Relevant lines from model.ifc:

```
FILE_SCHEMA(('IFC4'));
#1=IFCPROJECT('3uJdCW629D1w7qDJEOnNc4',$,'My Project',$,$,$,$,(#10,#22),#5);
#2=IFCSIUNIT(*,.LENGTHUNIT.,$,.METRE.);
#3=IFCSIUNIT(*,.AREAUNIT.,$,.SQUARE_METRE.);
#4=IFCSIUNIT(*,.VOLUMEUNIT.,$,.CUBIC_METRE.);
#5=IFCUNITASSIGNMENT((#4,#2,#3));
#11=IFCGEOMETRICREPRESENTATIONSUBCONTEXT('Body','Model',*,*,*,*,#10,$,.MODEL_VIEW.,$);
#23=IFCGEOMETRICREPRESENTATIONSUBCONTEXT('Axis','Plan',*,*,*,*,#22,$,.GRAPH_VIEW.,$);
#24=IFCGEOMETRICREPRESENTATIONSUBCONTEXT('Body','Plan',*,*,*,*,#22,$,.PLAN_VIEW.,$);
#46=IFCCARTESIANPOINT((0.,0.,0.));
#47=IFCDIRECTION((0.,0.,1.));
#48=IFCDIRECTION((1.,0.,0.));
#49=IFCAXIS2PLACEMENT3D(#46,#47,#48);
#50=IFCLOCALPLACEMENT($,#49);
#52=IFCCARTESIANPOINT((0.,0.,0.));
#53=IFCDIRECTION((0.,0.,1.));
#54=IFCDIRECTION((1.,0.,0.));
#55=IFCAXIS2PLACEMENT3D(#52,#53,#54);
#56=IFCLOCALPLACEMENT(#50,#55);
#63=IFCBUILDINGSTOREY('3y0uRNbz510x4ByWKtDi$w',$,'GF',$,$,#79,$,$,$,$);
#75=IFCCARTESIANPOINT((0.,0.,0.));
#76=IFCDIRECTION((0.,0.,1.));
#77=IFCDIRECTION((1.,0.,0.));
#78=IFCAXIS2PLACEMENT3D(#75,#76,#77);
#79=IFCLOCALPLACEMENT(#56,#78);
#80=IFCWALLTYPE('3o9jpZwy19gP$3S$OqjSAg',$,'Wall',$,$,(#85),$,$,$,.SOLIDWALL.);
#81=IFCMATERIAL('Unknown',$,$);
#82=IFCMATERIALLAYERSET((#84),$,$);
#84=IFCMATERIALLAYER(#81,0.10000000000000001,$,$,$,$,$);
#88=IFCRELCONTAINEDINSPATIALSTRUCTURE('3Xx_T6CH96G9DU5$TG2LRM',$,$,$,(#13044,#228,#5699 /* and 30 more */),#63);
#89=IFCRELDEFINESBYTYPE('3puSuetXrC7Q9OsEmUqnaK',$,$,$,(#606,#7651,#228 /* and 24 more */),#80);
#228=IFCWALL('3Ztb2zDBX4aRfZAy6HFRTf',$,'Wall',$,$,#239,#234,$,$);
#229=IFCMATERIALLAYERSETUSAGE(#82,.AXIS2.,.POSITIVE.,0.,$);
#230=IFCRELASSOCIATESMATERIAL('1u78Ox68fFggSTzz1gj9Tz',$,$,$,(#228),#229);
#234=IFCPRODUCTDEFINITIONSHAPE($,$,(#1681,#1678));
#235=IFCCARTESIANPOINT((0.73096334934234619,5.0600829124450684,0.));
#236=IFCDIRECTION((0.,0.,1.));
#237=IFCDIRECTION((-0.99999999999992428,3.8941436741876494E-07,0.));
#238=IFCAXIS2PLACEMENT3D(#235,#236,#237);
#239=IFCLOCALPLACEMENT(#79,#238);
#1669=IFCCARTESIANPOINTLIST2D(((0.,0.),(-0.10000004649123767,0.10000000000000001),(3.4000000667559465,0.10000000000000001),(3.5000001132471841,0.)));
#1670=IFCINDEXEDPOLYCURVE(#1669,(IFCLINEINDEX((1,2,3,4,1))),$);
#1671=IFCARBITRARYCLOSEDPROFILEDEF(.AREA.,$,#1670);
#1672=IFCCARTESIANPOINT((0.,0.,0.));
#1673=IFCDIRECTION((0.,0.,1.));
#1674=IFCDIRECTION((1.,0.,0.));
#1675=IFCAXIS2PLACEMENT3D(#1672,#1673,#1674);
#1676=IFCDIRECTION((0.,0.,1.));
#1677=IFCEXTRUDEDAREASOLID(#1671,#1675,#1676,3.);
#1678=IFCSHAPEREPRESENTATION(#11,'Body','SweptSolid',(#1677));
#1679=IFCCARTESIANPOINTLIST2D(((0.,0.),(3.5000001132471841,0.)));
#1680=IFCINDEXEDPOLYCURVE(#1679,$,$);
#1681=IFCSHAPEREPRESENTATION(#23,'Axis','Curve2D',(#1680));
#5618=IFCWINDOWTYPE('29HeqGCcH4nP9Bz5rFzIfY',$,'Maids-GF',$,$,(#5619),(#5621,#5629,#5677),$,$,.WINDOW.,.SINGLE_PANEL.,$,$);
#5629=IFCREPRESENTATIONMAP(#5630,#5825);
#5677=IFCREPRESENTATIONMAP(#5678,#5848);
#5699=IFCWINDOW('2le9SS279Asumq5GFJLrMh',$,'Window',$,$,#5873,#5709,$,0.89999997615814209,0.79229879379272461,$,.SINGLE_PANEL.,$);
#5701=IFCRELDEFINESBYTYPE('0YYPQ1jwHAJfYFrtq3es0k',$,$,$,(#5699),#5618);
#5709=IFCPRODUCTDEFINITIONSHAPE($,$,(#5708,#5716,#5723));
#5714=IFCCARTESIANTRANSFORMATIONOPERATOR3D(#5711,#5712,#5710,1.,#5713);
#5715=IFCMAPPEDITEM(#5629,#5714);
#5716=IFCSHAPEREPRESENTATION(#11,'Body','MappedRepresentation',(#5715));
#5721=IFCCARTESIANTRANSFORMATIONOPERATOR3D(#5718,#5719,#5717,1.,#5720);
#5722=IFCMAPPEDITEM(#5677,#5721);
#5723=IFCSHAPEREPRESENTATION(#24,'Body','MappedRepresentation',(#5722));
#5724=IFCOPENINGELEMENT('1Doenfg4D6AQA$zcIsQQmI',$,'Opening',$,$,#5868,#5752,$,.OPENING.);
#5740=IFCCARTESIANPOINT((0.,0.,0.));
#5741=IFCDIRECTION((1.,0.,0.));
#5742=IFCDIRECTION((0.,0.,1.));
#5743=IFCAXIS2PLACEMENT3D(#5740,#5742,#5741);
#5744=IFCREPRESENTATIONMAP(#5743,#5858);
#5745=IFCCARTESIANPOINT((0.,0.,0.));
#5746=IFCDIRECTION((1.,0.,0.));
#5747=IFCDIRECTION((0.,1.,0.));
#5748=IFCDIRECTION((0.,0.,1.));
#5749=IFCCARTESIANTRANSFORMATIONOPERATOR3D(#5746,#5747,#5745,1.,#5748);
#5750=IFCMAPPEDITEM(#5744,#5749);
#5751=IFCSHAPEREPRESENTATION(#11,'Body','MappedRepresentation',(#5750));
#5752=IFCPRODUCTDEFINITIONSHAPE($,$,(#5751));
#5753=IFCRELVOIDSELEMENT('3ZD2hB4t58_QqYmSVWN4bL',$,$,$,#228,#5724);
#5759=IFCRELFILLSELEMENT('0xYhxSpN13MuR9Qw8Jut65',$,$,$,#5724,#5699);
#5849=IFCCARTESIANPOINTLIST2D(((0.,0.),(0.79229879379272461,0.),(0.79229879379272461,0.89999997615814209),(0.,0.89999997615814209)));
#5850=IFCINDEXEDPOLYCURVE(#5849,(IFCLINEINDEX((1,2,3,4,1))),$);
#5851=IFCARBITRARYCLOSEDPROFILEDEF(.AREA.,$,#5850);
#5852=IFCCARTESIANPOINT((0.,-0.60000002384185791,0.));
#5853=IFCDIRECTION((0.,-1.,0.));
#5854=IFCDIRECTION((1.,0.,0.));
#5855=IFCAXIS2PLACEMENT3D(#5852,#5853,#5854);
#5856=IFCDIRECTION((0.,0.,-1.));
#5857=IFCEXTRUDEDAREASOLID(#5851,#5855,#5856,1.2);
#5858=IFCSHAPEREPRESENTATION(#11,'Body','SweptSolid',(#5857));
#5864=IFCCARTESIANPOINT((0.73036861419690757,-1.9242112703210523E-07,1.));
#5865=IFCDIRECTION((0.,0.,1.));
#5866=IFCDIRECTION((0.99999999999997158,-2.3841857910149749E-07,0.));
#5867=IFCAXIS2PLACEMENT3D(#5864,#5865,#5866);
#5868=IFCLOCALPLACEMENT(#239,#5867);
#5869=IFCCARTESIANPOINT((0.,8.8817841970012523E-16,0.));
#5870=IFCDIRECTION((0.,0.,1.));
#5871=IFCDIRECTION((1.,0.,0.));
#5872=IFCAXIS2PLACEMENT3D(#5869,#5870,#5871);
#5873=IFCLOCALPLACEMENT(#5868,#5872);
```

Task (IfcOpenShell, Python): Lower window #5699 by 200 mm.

```python
import numpy as np
import ifcopenshell
import ifcopenshell.api.geometry
import ifcopenshell.util.placement
import ifcopenshell.util.unit

model = ifcopenshell.open("model.ifc")
unit_scale = ifcopenshell.util.unit.calculate_unit_scale(model)

window = model.by_guid("2le9SS279Asumq5GFJLrMh")
opening = window.FillsVoids[0].RelatingOpeningElement
dz = -0.2 / unit_scale

shift = np.array([0.0, 0.0, dz])
# The window is placed relative to its opening, so it follows when the opening moves.
matrix = ifcopenshell.util.placement.get_local_placement(opening.ObjectPlacement)
matrix[:3, 3] += shift
ifcopenshell.api.geometry.edit_object_placement(
    model, product=opening, matrix=matrix, is_si=False, should_transform_children=True
)

print(f"moved by {dz * unit_scale:+.3f} m")

model.write("model_updated.ifc")
```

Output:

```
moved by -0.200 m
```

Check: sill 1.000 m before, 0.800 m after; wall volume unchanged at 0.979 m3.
